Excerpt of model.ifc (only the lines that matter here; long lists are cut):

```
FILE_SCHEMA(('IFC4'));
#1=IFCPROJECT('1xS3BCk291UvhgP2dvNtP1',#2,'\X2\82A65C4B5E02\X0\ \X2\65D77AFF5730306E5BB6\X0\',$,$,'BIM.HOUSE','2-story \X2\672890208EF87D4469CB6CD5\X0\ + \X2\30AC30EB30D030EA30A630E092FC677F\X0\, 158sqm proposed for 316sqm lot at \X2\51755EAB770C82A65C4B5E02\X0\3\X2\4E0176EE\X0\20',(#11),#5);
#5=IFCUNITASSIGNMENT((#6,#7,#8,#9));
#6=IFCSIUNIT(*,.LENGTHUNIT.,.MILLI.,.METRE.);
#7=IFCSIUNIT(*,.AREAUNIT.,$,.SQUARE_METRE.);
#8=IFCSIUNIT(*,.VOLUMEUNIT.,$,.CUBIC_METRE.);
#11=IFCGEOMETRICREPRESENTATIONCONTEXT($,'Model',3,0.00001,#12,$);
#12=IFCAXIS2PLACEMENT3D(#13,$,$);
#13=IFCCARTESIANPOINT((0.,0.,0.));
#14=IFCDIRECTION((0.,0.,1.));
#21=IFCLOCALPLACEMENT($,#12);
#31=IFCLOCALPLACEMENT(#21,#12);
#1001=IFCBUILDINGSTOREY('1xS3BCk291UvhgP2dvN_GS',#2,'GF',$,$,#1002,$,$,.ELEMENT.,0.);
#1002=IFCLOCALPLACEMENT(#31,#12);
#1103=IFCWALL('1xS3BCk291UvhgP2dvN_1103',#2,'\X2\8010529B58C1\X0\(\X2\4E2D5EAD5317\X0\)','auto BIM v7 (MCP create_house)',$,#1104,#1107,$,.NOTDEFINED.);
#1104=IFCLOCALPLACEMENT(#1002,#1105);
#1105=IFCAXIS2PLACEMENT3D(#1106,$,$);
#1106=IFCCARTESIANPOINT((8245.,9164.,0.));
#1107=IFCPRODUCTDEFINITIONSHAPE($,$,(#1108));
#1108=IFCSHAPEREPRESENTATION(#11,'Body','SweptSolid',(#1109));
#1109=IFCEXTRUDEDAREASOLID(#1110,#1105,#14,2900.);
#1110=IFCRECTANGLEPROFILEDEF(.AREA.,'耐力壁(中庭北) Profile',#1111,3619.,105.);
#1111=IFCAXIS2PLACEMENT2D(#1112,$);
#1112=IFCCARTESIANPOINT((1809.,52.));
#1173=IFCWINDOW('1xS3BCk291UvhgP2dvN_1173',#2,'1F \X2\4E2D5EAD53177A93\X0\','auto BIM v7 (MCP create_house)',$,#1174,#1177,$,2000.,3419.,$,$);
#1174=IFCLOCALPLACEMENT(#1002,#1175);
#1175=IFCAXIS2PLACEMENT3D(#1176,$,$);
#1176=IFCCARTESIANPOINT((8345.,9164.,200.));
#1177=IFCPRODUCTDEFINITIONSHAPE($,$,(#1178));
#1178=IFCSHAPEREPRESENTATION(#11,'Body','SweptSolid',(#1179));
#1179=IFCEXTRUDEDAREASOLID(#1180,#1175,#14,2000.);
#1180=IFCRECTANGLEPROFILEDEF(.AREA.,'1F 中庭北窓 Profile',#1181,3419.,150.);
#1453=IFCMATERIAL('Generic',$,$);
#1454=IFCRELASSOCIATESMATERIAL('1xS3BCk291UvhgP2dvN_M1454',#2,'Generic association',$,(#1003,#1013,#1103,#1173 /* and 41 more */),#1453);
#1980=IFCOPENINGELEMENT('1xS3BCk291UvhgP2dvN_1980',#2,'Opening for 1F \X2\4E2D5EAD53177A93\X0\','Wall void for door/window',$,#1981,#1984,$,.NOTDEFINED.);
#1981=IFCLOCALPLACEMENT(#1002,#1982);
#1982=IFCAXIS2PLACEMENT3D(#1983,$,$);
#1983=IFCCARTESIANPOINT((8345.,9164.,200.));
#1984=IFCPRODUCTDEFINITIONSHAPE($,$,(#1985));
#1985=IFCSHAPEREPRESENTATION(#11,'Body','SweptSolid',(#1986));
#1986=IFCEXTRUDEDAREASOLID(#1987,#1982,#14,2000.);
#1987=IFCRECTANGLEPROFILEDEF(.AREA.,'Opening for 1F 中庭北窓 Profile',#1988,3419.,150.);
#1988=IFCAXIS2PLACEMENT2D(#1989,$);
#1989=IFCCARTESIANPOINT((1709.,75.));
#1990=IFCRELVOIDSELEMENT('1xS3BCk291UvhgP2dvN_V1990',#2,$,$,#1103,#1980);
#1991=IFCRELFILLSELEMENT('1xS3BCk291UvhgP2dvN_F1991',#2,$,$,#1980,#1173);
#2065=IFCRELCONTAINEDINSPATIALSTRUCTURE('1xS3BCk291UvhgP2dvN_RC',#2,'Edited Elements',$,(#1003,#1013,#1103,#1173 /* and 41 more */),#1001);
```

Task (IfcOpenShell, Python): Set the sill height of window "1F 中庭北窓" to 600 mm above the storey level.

```python
import numpy as np
import ifcopenshell
import ifcopenshell.api.geometry
import ifcopenshell.geom
import ifcopenshell.util.element
import ifcopenshell.util.placement
import ifcopenshell.util.shape
import ifcopenshell.util.unit

model = ifcopenshell.open("model.ifc")
unit_scale = ifcopenshell.util.unit.calculate_unit_scale(model)

window = model.by_guid("1xS3BCk291UvhgP2dvN_1173")
opening = window.FillsVoids[0].RelatingOpeningElement
storey = ifcopenshell.util.element.get_container(window, ifc_class="IfcBuildingStorey")
level = ifcopenshell.util.placement.get_local_placement(storey.ObjectPlacement)[2, 3]

# The opening's origin need not be at the sill, so measure its lowest point.
shape = ifcopenshell.geom.create_shape(ifcopenshell.geom.settings(), opening)
bottom = ifcopenshell.util.shape.get_shape_bottom_elevation(shape, shape.geometry) / unit_scale
dz = level + 600.0 - bottom

shift = np.array([0.0, 0.0, dz])
# The window is not placed relative to its opening, so move both.
for product in (opening, window):
    matrix = ifcopenshell.util.placement.get_local_placement(product.ObjectPlacement)
    matrix[:3, 3] += shift
    ifcopenshell.api.geometry.edit_object_placement(model, product=product, matrix=matrix, is_si=False)

print(f"moved by {dz * unit_scale:+.3f} m")

model.write("model-out.ifc")
```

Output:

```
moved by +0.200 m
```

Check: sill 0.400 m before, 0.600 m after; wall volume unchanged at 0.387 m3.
